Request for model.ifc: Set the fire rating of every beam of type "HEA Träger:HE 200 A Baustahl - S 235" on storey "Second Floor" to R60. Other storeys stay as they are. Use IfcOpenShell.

First a look at what the model holds.

```python
import ifcopenshell
import ifcopenshell.util.element

model = ifcopenshell.open("model.ifc")
print(model.schema)
storey = next(s for s in model.by_type("IfcBuildingStorey") if s.Name == "Second Floor")
beams = [e for e in ifcopenshell.util.element.get_decomposition(storey) if e.is_a("IfcBeam")]
seen = {}
for e in beams:
    element_type = ifcopenshell.util.element.get_type(e)
    key = (element_type.Name if element_type != e and element_type else None, ifcopenshell.util.element.get_pset(e, "Pset_BeamCommon", "FireRating"))
    seen[key] = seen.get(key, 0) + 1
for (name, value), count in sorted(seen.items(), key=str):
    print(count, "x", name, "|", value)
```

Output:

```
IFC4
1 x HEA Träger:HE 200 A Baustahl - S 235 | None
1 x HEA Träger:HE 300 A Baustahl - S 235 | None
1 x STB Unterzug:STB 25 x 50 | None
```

```python
import ifcopenshell
import ifcopenshell.api.pset
import ifcopenshell.util.element

model = ifcopenshell.open("model.ifc")

storey = next(s for s in model.by_type("IfcBuildingStorey") if s.Name == "Second Floor")
beams = [e for e in ifcopenshell.util.element.get_decomposition(storey) if e.is_a("IfcBeam")]

count = 0
for e in beams:
    element_type = ifcopenshell.util.element.get_type(e)
    if element_type in (None, e) or element_type.Name != "HEA Träger:HE 200 A Baustahl - S 235":
        continue
    # add_pset returns the element's existing set when there is one.
    pset = ifcopenshell.api.pset.add_pset(model, product=e, name="Pset_BeamCommon")
    ifcopenshell.api.pset.edit_pset(model, pset=pset, properties={"FireRating": "R60"})
    count += 1

print(count, "beams updated")

model.write("model_updated.ifc")
```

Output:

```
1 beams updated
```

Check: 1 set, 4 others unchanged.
